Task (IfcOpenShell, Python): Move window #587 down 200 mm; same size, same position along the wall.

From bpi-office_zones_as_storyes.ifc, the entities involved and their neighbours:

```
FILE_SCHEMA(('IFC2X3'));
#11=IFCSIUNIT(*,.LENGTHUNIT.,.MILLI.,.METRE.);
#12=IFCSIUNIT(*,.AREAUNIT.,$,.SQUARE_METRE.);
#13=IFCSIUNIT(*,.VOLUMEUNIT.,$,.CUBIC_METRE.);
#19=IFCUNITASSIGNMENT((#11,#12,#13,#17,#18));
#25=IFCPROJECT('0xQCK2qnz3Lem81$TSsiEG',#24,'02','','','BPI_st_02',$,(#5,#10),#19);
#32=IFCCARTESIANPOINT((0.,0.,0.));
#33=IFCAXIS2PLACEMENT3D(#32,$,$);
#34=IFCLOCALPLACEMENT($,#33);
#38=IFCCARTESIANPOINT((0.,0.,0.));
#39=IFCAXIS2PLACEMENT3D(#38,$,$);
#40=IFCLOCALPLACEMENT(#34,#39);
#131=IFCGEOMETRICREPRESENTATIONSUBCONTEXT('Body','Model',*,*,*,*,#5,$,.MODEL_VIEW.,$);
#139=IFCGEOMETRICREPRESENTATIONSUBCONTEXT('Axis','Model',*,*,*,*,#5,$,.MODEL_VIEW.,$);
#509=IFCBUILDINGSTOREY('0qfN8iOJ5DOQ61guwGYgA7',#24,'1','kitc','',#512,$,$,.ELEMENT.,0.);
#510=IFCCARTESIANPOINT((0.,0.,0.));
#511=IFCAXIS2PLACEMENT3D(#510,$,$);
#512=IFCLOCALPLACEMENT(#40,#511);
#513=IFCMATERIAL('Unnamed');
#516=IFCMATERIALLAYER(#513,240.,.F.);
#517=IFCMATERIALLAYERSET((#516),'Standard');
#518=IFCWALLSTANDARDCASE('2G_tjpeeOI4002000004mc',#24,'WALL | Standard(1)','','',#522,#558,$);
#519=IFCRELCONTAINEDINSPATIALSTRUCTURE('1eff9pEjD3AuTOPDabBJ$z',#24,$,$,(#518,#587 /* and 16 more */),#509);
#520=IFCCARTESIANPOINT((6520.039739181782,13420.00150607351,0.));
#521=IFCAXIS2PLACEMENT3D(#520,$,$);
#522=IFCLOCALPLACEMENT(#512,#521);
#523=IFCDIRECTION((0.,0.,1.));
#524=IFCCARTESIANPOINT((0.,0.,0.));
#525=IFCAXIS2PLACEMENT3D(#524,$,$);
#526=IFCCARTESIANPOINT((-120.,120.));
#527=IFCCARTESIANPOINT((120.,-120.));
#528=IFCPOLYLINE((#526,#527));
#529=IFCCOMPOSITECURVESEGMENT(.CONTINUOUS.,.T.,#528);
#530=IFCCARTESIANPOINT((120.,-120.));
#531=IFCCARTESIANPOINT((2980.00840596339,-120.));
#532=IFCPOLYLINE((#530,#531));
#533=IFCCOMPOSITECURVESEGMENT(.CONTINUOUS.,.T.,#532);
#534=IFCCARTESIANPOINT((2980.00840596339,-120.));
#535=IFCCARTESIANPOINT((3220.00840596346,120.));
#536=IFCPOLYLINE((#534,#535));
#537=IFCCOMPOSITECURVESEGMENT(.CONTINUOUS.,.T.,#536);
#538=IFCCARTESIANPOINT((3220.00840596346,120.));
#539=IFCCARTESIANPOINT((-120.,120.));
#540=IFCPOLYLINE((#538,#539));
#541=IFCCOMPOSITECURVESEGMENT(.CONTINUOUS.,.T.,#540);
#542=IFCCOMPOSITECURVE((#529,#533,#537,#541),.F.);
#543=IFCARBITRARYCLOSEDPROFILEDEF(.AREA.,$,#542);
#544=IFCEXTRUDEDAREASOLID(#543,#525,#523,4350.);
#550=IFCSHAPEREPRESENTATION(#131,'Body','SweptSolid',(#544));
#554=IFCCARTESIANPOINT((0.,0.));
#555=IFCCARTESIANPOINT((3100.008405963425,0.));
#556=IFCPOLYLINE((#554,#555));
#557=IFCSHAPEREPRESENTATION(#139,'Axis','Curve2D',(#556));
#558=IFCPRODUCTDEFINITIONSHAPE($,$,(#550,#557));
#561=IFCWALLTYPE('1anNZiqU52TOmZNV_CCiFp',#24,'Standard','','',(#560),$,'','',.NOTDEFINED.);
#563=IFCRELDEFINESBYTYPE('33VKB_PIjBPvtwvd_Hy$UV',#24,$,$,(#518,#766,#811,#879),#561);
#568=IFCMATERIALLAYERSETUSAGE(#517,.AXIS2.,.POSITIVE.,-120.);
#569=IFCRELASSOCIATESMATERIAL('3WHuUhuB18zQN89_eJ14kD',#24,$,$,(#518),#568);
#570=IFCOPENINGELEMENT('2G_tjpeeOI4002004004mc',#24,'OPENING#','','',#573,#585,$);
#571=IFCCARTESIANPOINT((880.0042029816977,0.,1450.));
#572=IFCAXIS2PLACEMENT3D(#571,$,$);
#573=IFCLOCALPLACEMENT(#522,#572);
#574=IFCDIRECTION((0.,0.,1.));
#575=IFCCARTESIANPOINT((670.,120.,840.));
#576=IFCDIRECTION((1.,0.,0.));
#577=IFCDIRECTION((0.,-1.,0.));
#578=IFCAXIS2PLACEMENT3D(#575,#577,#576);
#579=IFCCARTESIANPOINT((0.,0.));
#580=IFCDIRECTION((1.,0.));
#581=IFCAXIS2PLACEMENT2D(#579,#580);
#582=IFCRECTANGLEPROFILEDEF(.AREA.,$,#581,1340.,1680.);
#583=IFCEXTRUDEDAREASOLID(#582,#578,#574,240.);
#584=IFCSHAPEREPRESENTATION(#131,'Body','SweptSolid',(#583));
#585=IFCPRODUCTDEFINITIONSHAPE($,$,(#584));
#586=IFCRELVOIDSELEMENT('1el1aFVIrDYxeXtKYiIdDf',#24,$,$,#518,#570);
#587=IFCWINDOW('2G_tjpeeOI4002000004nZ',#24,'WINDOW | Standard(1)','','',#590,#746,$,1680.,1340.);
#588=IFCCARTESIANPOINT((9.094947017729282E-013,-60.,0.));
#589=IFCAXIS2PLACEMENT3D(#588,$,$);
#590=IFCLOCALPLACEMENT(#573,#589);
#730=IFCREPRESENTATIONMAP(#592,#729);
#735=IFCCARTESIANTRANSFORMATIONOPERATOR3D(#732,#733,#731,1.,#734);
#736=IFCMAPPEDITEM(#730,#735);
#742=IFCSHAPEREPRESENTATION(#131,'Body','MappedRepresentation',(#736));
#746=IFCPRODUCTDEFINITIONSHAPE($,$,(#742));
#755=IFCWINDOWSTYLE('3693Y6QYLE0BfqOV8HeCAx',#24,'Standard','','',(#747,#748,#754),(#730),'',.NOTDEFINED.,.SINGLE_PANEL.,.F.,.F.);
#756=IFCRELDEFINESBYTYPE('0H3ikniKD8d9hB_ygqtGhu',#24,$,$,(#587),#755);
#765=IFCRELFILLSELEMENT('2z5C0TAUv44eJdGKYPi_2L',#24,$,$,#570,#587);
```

```python
import numpy as np
import ifcopenshell
import ifcopenshell.api.geometry
import ifcopenshell.util.placement
import ifcopenshell.util.unit

model = ifcopenshell.open("bpi-office_zones_as_storyes.ifc")
unit_scale = ifcopenshell.util.unit.calculate_unit_scale(model)

window = model.by_id(587)
opening = window.FillsVoids[0].RelatingOpeningElement
dz = -0.2 / unit_scale

shift = np.array([0.0, 0.0, dz])
# The window is placed relative to its opening, so it follows when the opening moves.
matrix = ifcopenshell.util.placement.get_local_placement(opening.ObjectPlacement)
matrix[:3, 3] += shift
ifcopenshell.api.geometry.edit_object_placement(
    model, product=opening, matrix=matrix, is_si=False, should_transform_children=True
)

print(f"moved by {dz * unit_scale:+.3f} m")

model.write("bpi-office_zones_as_storyes_v2.ifc")
```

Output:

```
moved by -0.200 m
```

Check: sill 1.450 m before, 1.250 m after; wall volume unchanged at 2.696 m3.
